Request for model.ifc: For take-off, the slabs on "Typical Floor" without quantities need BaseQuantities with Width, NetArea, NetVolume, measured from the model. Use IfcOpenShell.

First a look at what the model holds.

```python
import ifcopenshell
import ifcopenshell.util.element
import ifcopenshell.util.unit

model = ifcopenshell.open("model.ifc")
print(model.schema)
for unit_type in ("LENGTHUNIT", "AREAUNIT", "VOLUMEUNIT"):
    print(unit_type, ifcopenshell.util.unit.calculate_unit_scale(model, unit_type))
storey = next(s for s in model.by_type("IfcBuildingStorey") if s.Name == "Typical Floor")
slabs = [e for e in ifcopenshell.util.element.get_decomposition(storey) if e.is_a("IfcSlab")]
for e in sorted(slabs, key=lambda e: e.id()):
    print(e.id(), e.is_a(), e.Name, list(ifcopenshell.util.element.get_psets(e, qtos_only=True)), sep=" | ")
```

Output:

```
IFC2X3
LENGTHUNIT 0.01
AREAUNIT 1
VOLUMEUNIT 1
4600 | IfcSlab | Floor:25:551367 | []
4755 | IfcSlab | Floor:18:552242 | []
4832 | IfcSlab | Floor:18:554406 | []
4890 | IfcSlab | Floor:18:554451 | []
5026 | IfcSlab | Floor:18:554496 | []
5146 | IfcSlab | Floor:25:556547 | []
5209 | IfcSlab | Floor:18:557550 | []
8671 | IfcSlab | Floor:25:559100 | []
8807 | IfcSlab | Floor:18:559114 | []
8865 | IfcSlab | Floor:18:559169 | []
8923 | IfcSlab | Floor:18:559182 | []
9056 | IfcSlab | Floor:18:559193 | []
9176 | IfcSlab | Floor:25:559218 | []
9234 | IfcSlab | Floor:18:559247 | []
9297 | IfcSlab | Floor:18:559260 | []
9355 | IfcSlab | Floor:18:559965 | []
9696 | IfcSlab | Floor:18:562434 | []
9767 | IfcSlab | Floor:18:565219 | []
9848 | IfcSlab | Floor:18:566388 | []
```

```python
import ifcopenshell
import ifcopenshell.api.pset
import ifcopenshell.geom
import ifcopenshell.util.element
import ifcopenshell.util.shape
import ifcopenshell.util.unit

model = ifcopenshell.open("model.ifc")
unit_scale = ifcopenshell.util.unit.calculate_unit_scale(model)
area_scale = ifcopenshell.util.unit.calculate_unit_scale(model, "AREAUNIT")
volume_scale = ifcopenshell.util.unit.calculate_unit_scale(model, "VOLUMEUNIT")
settings = ifcopenshell.geom.settings()

storey = next(s for s in model.by_type("IfcBuildingStorey") if s.Name == "Typical Floor")
slabs = [e for e in ifcopenshell.util.element.get_decomposition(storey) if e.is_a("IfcSlab")]

for e in sorted(slabs, key=lambda e: e.id()):
    if ifcopenshell.util.element.get_psets(e, qtos_only=True, should_inherit=False):
        continue
    # Geometry comes back in metres, in the element's own axes.
    shape = ifcopenshell.geom.create_shape(settings, e)
    values = {
        "Width": ifcopenshell.util.shape.get_z(shape.geometry) / unit_scale,
        "NetArea": ifcopenshell.util.shape.get_footprint_area(shape.geometry) / area_scale,
        "NetVolume": ifcopenshell.util.shape.get_volume(shape.geometry) / volume_scale,
    }
    qto = ifcopenshell.api.pset.add_qto(model, product=e, name="BaseQuantities")
    ifcopenshell.api.pset.edit_qto(model, qto=qto, properties=values)
    print(e.id(), {k: round(v, 3) for k, v in values.items()})

model.write("model_rev.ifc")
```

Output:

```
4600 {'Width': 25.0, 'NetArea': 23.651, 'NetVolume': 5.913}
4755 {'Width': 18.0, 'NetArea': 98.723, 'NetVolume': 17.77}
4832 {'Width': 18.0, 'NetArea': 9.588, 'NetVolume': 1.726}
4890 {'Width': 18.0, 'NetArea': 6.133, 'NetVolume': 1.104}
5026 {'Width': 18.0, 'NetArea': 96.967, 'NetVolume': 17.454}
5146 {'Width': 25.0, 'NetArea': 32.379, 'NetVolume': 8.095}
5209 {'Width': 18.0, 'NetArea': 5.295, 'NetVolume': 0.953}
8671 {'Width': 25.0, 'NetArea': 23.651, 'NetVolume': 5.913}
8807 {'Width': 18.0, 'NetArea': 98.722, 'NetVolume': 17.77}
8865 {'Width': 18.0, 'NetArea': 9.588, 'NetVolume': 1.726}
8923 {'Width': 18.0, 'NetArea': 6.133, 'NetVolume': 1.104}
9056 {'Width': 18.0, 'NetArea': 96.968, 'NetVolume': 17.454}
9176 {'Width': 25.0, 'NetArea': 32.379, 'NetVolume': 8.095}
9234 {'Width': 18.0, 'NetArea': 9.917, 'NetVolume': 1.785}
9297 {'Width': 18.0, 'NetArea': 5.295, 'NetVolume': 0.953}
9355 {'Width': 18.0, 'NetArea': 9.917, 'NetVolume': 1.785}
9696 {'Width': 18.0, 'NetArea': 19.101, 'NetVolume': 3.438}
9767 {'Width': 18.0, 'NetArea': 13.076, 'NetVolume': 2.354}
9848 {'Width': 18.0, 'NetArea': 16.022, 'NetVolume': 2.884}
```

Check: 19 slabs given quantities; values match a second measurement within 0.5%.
